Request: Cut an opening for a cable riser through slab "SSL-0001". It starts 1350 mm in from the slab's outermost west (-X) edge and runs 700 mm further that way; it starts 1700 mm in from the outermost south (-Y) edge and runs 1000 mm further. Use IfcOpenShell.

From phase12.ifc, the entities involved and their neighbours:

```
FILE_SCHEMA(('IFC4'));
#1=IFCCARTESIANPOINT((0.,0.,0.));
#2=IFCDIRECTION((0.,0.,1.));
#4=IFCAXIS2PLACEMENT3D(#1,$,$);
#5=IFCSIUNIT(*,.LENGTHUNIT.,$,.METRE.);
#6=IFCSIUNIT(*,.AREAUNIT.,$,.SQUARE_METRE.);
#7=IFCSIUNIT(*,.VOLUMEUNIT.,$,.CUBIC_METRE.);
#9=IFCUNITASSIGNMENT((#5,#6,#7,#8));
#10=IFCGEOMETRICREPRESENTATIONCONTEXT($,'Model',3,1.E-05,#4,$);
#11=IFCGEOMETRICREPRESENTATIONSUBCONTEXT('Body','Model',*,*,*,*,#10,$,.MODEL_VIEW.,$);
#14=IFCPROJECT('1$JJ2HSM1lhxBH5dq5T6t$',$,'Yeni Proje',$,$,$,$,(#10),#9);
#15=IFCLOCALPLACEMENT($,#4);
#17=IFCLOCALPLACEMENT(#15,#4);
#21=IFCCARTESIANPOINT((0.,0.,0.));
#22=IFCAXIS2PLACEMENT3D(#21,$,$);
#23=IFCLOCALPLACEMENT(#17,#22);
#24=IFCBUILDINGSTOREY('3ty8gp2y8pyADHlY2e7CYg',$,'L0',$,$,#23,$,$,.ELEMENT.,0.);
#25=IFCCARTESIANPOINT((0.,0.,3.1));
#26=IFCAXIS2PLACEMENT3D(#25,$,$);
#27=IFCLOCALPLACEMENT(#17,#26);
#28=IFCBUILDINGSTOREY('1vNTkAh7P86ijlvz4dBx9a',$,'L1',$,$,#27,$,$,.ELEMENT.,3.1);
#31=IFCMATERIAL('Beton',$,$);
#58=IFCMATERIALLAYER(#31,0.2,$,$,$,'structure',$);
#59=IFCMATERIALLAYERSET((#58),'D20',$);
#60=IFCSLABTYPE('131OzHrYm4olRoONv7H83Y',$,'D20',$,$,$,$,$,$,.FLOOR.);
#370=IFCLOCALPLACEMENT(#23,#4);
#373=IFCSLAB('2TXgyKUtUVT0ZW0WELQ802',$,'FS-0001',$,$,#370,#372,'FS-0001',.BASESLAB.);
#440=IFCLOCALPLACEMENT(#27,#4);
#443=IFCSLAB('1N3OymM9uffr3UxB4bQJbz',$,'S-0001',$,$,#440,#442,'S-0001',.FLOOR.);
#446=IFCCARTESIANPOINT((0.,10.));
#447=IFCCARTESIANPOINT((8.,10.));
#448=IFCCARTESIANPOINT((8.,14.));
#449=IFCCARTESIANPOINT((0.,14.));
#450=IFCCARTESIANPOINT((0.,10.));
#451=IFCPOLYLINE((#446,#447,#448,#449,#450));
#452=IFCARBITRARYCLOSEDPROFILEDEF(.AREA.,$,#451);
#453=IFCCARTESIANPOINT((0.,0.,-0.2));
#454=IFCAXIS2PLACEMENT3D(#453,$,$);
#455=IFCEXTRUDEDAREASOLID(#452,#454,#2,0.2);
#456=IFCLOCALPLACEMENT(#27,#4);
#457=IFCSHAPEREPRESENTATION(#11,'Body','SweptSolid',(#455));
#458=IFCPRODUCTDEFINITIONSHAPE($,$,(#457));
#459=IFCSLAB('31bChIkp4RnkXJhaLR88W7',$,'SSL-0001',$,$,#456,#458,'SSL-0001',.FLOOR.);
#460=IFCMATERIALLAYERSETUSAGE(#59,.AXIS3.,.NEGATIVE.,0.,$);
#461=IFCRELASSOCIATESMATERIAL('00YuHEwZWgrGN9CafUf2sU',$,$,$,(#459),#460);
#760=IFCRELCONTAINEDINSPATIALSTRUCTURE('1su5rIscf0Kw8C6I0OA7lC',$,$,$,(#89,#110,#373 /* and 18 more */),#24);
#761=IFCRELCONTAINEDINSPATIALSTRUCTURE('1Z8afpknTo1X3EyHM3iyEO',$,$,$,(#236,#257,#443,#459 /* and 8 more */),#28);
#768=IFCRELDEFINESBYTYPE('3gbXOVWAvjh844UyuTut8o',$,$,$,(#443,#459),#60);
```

```python
import numpy as np
import ifcopenshell
import ifcopenshell.api.feature
import ifcopenshell.api.geometry
import ifcopenshell.api.root
import ifcopenshell.geom
import ifcopenshell.util.placement
import ifcopenshell.util.representation
import ifcopenshell.util.shape
import ifcopenshell.util.unit

model = ifcopenshell.open("phase12.ifc")
unit_scale = ifcopenshell.util.unit.calculate_unit_scale(model)
settings = ifcopenshell.geom.settings()


def volume(element):
    """Net volume in cubic metres, openings subtracted."""
    shape = ifcopenshell.geom.create_shape(settings, element)
    return ifcopenshell.util.shape.get_volume(shape.geometry)


slab = model.by_id(459)
before = volume(slab)

# Extent in the slab's own axes, in metres. The edges named are its -X and -Y sides.
slab_shape = ifcopenshell.geom.create_shape(settings, slab)
vertices = ifcopenshell.util.shape.get_vertices(slab_shape.geometry)
x_min, y_min, bottom = vertices.min(axis=0)
top = vertices[:, 2].max()

opening = ifcopenshell.api.root.create_entity(model, ifc_class="IfcOpeningElement", name="Cable riser opening", predefined_type="OPENING")
context = ifcopenshell.util.representation.get_context(model, "Model", "Body", "MODEL_VIEW")
width, depth = 0.7, 1
outline = [(0.0, 0.0), (width, 0.0), (width, depth), (0.0, depth), (0.0, 0.0)]
# Overshoot both faces by 50 mm so the cut is clean.
shape = ifcopenshell.api.geometry.add_slab_representation(
    model, context=context, depth=top - bottom + 0.1, polyline=outline
)
ifcopenshell.api.geometry.assign_representation(model, product=opening, representation=shape)

matrix = ifcopenshell.util.placement.get_local_placement(slab.ObjectPlacement)
matrix[:, 3] = matrix @ np.append(np.array([x_min + 1.35, y_min + 1.7, bottom - 0.05]) / unit_scale, 1.0)
ifcopenshell.api.geometry.edit_object_placement(model, product=opening, matrix=matrix, is_si=False)
ifcopenshell.api.feature.add_feature(model, feature=opening, element=slab)

after = volume(slab)

print(f"slab volume {before:.3f} -> {after:.3f} m3")

model.write("phase12_rev.ifc")
```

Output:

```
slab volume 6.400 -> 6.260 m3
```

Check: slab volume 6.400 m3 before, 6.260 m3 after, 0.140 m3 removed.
